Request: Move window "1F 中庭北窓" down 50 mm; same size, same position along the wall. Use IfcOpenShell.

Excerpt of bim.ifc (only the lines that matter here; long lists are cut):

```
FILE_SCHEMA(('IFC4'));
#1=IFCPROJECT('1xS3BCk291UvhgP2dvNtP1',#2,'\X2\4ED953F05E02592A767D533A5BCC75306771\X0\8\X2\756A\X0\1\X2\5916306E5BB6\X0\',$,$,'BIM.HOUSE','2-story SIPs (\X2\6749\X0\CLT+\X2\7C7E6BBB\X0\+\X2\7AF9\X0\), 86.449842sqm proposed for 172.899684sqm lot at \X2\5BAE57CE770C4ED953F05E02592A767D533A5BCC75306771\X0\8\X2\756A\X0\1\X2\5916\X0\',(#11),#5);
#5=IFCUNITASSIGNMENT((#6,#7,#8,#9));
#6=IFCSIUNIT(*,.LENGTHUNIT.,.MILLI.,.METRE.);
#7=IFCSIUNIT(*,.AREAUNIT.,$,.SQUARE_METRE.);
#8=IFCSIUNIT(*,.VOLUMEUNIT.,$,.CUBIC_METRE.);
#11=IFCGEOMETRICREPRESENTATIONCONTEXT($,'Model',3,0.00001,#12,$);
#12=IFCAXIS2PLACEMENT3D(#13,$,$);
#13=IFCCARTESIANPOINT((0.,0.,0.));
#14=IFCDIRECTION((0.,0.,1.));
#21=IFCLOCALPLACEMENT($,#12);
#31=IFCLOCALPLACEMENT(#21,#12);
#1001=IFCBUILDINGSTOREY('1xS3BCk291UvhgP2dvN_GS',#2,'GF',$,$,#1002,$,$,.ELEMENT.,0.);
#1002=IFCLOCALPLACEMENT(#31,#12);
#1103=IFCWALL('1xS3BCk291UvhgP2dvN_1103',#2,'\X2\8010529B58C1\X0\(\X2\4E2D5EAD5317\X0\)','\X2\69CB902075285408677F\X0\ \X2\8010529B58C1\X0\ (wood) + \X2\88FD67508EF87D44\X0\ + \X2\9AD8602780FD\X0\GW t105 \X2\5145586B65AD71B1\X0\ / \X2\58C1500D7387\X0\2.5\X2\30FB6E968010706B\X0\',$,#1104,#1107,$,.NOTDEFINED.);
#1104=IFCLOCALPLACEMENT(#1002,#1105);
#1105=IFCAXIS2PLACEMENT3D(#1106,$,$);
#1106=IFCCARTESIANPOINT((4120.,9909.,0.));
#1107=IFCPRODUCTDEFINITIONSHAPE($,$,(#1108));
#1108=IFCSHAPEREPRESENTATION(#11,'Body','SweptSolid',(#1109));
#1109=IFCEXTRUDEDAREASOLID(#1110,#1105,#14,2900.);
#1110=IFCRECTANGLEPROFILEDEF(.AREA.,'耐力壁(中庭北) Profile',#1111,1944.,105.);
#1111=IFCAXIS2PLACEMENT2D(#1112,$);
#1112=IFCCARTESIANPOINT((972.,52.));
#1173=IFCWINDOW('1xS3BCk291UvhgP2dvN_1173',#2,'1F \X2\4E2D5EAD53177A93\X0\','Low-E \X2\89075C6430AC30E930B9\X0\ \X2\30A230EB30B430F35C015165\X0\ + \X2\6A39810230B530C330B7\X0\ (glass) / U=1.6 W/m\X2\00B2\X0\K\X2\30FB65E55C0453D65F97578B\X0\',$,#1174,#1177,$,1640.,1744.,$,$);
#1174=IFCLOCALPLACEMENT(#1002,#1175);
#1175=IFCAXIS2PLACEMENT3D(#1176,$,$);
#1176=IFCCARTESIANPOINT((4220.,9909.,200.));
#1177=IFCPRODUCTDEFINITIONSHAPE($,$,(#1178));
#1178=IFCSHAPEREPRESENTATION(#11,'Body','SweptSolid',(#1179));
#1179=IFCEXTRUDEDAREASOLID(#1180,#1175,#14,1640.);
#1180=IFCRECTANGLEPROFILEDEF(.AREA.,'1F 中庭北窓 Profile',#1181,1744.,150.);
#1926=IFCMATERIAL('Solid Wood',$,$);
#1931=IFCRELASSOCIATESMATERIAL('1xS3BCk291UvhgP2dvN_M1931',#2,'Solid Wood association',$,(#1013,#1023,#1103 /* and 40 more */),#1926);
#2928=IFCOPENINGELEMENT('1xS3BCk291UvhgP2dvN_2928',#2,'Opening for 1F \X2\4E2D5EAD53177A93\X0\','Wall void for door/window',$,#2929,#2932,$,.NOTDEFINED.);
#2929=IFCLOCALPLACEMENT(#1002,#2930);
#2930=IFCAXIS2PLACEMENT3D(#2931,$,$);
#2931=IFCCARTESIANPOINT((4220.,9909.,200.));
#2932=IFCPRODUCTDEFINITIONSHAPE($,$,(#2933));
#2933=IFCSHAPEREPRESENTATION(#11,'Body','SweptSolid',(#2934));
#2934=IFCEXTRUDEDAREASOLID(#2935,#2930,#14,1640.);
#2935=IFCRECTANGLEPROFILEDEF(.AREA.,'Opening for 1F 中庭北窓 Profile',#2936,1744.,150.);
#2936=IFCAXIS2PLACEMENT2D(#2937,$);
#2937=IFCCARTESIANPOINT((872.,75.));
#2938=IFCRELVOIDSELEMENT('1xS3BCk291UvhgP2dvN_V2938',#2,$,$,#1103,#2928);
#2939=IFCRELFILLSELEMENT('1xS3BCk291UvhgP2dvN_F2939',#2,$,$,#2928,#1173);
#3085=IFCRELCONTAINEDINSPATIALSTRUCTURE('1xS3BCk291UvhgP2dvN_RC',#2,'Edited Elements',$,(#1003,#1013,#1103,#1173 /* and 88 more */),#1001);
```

```python
import numpy as np
import ifcopenshell
import ifcopenshell.api.geometry
import ifcopenshell.util.placement
import ifcopenshell.util.unit

model = ifcopenshell.open("bim.ifc")
unit_scale = ifcopenshell.util.unit.calculate_unit_scale(model)

window = model.by_guid("1xS3BCk291UvhgP2dvN_1173")
opening = window.FillsVoids[0].RelatingOpeningElement
dz = -50.0

shift = np.array([0.0, 0.0, dz])
# The window is not placed relative to its opening, so move both.
for product in (opening, window):
    matrix = ifcopenshell.util.placement.get_local_placement(product.ObjectPlacement)
    matrix[:3, 3] += shift
    ifcopenshell.api.geometry.edit_object_placement(model, product=product, matrix=matrix, is_si=False)

print(f"moved by {dz * unit_scale:+.3f} m")

model.write("bim_edited.ifc")
```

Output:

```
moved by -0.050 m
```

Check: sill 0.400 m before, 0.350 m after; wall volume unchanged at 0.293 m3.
